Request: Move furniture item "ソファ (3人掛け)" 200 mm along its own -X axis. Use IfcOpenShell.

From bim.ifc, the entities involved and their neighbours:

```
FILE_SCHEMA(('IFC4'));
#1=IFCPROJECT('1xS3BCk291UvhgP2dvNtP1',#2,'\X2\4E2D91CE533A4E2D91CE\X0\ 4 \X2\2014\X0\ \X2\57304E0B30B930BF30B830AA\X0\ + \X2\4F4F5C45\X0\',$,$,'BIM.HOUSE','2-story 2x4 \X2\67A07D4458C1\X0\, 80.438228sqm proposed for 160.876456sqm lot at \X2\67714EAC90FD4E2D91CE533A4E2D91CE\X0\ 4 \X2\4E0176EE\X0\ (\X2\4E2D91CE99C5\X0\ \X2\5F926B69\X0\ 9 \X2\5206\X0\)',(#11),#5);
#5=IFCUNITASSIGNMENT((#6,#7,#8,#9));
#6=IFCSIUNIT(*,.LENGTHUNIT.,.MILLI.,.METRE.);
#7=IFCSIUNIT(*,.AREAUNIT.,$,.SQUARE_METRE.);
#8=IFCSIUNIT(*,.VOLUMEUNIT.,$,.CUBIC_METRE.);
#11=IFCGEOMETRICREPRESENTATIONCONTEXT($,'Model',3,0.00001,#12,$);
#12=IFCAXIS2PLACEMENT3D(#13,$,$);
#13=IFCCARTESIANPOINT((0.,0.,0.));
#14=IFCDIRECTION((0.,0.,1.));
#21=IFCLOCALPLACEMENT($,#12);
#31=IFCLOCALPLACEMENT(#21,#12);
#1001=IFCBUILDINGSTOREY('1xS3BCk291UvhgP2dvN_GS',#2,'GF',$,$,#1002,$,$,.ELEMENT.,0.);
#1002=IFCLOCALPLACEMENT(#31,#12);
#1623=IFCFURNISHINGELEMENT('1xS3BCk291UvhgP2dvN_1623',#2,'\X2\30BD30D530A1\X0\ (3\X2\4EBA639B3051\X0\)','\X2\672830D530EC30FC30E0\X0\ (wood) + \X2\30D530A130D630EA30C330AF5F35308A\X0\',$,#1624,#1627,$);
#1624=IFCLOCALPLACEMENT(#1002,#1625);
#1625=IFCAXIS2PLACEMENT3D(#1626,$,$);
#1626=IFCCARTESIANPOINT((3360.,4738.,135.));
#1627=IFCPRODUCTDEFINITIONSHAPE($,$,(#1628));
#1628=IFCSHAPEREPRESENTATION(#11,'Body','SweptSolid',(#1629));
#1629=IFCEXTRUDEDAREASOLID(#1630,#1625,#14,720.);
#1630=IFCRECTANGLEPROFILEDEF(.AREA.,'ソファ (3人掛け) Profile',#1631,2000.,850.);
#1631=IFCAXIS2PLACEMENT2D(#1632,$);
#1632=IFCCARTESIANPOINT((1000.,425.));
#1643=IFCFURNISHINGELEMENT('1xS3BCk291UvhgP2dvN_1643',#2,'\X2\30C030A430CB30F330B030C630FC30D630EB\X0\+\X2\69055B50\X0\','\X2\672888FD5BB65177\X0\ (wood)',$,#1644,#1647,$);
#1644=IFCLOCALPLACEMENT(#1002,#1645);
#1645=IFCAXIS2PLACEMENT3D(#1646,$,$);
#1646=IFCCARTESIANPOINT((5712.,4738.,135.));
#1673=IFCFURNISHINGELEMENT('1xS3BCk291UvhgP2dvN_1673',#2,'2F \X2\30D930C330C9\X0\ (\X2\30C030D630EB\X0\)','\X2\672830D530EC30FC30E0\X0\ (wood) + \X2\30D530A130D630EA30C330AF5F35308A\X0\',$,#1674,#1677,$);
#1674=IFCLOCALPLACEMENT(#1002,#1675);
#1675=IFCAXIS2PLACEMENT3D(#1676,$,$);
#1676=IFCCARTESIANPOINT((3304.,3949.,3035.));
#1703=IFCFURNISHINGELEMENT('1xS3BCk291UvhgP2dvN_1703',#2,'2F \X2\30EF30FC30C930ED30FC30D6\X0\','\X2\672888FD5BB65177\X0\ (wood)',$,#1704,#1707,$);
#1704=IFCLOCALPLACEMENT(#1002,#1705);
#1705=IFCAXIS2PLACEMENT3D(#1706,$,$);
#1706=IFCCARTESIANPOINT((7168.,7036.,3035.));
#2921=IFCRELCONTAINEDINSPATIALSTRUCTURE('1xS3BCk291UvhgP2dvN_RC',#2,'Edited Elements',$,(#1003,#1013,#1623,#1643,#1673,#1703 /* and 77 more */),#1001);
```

```python
import ifcopenshell
import ifcopenshell.api.geometry
import ifcopenshell.util.placement

model = ifcopenshell.open("bim.ifc")

item = model.by_id(1623)
matrix = ifcopenshell.util.placement.get_local_placement(item.ObjectPlacement)
matrix[:3, 3] -= matrix[:3, 0] * 200.0
ifcopenshell.api.geometry.edit_object_placement(model, product=item, matrix=matrix, is_si=False)

print(ifcopenshell.util.placement.get_local_placement(item.ObjectPlacement).round(3) + 0.0)

model.write("bim-out.ifc")
```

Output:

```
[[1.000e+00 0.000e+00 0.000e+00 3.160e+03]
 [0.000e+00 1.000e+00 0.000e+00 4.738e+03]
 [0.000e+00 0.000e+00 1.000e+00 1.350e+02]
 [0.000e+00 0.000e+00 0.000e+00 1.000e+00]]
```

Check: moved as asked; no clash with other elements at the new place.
